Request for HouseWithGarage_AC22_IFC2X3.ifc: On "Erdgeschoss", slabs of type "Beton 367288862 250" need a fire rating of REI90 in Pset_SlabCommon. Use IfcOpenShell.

First a look at what the model holds.

```python
import ifcopenshell
import ifcopenshell.util.element

model = ifcopenshell.open("HouseWithGarage_AC22_IFC2X3.ifc")
print(model.schema)
storey = next(s for s in model.by_type("IfcBuildingStorey") if s.Name == "Erdgeschoss")
slabs = [e for e in ifcopenshell.util.element.get_decomposition(storey) if e.is_a("IfcSlab")]
seen = {}
for e in slabs:
    element_type = ifcopenshell.util.element.get_type(e)
    key = (element_type.Name if element_type != e and element_type else None, ifcopenshell.util.element.get_pset(e, "Pset_SlabCommon", "FireRating"))
    seen[key] = seen.get(key, 0) + 1
for (name, value), count in sorted(seen.items(), key=str):
    print(count, "x", name, "|", value)
```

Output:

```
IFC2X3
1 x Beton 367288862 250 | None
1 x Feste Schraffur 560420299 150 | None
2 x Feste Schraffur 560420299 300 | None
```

```python
import ifcopenshell
import ifcopenshell.api.pset
import ifcopenshell.util.element

model = ifcopenshell.open("HouseWithGarage_AC22_IFC2X3.ifc")

storey = next(s for s in model.by_type("IfcBuildingStorey") if s.Name == "Erdgeschoss")
slabs = [e for e in ifcopenshell.util.element.get_decomposition(storey) if e.is_a("IfcSlab")]

count = 0
for e in slabs:
    element_type = ifcopenshell.util.element.get_type(e)
    if element_type in (None, e) or element_type.Name != "Beton 367288862 250":
        continue
    # add_pset returns the element's existing set when there is one.
    pset = ifcopenshell.api.pset.add_pset(model, product=e, name="Pset_SlabCommon")
    ifcopenshell.api.pset.edit_pset(model, pset=pset, properties={"FireRating": "REI90"})
    count += 1

print(count, "slabs updated")

model.write("HouseWithGarage_AC22_IFC2X3_v2.ifc")
```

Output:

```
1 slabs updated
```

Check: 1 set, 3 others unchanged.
